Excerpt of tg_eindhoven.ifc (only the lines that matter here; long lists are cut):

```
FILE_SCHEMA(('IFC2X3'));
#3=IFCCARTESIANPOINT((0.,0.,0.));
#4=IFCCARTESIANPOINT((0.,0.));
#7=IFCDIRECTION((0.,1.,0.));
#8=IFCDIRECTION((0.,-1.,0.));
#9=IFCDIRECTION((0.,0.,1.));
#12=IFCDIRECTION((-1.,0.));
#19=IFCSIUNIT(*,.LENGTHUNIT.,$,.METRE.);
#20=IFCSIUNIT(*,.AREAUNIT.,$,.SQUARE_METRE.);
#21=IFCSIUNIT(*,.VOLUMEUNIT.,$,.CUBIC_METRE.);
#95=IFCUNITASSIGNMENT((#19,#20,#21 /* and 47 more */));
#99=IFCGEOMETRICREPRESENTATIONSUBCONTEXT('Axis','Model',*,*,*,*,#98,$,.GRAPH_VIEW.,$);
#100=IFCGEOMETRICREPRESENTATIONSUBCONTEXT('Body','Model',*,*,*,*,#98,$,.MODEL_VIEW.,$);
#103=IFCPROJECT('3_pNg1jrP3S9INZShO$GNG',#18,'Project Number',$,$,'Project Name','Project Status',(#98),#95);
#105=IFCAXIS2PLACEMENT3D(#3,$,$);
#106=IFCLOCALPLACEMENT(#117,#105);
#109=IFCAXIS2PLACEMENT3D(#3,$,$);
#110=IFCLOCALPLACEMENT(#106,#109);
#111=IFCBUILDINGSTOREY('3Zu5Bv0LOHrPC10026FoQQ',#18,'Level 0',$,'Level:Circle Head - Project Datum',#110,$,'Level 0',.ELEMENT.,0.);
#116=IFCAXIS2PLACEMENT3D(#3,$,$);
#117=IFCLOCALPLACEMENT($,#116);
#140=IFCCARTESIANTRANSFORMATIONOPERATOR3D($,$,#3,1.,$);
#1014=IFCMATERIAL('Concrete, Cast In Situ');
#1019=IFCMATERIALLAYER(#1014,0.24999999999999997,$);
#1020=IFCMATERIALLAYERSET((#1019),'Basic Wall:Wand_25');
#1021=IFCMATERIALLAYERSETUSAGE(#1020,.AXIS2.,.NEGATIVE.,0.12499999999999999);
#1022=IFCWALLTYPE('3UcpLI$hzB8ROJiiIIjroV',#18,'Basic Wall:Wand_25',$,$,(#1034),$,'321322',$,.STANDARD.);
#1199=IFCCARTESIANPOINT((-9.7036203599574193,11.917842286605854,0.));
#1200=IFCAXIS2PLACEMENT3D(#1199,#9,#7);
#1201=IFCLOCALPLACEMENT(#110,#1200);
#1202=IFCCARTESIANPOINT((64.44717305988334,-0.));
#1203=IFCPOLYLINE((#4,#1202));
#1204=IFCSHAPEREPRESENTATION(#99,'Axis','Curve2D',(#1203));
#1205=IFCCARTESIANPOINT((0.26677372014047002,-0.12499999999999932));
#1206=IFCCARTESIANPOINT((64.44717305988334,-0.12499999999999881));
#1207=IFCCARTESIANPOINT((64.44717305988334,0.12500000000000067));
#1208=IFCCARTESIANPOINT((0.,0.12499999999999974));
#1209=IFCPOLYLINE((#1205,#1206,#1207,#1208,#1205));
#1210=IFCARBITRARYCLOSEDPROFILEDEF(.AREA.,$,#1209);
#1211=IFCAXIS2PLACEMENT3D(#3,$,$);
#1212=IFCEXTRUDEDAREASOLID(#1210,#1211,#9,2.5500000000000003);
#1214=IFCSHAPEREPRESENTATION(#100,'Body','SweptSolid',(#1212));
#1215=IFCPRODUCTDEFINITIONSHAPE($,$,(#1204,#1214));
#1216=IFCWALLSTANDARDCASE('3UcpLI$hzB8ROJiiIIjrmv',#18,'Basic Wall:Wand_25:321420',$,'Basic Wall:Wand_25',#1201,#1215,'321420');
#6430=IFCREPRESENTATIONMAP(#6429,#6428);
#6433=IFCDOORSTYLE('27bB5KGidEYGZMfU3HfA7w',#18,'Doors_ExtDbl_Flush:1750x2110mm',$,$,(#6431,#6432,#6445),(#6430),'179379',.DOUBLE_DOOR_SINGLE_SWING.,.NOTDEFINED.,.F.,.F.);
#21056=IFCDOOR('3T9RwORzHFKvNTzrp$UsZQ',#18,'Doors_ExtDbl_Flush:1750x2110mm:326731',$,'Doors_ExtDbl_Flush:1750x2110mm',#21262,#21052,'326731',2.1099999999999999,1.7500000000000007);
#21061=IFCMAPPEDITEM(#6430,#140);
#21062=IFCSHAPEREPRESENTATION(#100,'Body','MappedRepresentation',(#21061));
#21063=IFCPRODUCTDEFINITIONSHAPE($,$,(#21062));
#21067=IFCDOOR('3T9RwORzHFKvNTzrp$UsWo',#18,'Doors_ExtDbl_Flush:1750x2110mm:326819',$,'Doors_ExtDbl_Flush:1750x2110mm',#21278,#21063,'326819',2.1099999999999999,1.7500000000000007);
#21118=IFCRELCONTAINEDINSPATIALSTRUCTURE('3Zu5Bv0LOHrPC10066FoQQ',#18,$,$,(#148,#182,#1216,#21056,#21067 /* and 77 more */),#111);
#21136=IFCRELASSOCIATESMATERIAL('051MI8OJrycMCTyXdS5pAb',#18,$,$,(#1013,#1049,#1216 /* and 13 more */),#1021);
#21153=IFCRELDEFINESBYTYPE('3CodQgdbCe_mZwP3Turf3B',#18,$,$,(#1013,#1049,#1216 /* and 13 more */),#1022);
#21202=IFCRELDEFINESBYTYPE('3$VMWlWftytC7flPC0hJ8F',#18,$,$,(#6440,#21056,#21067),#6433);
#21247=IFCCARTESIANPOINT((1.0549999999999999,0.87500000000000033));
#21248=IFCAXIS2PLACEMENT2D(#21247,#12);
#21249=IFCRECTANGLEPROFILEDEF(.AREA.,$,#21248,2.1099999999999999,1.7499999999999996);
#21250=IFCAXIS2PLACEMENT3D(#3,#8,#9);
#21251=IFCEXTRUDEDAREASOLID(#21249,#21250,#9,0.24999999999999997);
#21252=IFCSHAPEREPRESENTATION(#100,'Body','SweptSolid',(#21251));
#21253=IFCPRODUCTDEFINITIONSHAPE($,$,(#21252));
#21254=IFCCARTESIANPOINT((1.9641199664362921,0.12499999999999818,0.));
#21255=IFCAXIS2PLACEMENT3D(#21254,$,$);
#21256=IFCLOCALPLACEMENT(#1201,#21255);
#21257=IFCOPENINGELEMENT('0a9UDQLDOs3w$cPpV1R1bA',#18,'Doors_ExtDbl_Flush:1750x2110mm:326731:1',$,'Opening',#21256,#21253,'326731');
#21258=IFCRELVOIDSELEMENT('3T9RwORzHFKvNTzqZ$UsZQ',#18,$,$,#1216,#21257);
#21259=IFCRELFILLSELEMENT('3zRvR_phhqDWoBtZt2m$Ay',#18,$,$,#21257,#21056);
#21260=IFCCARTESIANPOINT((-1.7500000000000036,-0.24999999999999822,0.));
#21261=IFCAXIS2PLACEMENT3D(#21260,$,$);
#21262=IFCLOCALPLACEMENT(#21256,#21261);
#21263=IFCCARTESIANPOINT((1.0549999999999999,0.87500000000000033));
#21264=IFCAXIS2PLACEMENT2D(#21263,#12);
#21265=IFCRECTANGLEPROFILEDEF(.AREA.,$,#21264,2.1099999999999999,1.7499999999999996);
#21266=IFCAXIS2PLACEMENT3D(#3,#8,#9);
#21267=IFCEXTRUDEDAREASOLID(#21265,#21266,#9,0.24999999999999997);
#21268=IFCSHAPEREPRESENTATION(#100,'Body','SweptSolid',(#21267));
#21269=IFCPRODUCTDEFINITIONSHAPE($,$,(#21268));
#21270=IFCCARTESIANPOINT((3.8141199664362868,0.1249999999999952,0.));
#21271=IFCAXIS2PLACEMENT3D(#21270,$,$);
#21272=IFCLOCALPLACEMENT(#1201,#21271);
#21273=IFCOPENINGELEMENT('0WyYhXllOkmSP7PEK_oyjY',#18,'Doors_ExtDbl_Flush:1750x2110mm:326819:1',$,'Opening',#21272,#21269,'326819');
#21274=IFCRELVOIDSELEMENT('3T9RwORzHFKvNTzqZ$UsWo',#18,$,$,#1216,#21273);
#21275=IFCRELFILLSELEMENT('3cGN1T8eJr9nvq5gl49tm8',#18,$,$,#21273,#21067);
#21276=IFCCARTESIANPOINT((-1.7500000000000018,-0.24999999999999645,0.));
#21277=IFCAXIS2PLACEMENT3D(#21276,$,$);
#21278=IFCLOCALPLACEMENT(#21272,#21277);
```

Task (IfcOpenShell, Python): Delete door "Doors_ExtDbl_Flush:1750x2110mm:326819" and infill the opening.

```python
import ifcopenshell
import ifcopenshell.api.feature
import ifcopenshell.api.root
import ifcopenshell.geom
import ifcopenshell.util.shape

model = ifcopenshell.open("tg_eindhoven.ifc")
settings = ifcopenshell.geom.settings()


def volume(element):
    """Net volume in cubic metres, openings subtracted."""
    shape = ifcopenshell.geom.create_shape(settings, element)
    return ifcopenshell.util.shape.get_volume(shape.geometry)


door = model.by_id(21067)
opening = door.FillsVoids[0].RelatingOpeningElement
wall = opening.VoidsElements[0].RelatingBuildingElement
before = volume(wall)

ifcopenshell.api.root.remove_product(model, product=door)
ifcopenshell.api.feature.remove_feature(model, feature=opening)

after = volume(wall)

print(f"wall volume {before:.3f} -> {after:.3f} m3")

model.write("tg_eindhoven_v2.ifc")
```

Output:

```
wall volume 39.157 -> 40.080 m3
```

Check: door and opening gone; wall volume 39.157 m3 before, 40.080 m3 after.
